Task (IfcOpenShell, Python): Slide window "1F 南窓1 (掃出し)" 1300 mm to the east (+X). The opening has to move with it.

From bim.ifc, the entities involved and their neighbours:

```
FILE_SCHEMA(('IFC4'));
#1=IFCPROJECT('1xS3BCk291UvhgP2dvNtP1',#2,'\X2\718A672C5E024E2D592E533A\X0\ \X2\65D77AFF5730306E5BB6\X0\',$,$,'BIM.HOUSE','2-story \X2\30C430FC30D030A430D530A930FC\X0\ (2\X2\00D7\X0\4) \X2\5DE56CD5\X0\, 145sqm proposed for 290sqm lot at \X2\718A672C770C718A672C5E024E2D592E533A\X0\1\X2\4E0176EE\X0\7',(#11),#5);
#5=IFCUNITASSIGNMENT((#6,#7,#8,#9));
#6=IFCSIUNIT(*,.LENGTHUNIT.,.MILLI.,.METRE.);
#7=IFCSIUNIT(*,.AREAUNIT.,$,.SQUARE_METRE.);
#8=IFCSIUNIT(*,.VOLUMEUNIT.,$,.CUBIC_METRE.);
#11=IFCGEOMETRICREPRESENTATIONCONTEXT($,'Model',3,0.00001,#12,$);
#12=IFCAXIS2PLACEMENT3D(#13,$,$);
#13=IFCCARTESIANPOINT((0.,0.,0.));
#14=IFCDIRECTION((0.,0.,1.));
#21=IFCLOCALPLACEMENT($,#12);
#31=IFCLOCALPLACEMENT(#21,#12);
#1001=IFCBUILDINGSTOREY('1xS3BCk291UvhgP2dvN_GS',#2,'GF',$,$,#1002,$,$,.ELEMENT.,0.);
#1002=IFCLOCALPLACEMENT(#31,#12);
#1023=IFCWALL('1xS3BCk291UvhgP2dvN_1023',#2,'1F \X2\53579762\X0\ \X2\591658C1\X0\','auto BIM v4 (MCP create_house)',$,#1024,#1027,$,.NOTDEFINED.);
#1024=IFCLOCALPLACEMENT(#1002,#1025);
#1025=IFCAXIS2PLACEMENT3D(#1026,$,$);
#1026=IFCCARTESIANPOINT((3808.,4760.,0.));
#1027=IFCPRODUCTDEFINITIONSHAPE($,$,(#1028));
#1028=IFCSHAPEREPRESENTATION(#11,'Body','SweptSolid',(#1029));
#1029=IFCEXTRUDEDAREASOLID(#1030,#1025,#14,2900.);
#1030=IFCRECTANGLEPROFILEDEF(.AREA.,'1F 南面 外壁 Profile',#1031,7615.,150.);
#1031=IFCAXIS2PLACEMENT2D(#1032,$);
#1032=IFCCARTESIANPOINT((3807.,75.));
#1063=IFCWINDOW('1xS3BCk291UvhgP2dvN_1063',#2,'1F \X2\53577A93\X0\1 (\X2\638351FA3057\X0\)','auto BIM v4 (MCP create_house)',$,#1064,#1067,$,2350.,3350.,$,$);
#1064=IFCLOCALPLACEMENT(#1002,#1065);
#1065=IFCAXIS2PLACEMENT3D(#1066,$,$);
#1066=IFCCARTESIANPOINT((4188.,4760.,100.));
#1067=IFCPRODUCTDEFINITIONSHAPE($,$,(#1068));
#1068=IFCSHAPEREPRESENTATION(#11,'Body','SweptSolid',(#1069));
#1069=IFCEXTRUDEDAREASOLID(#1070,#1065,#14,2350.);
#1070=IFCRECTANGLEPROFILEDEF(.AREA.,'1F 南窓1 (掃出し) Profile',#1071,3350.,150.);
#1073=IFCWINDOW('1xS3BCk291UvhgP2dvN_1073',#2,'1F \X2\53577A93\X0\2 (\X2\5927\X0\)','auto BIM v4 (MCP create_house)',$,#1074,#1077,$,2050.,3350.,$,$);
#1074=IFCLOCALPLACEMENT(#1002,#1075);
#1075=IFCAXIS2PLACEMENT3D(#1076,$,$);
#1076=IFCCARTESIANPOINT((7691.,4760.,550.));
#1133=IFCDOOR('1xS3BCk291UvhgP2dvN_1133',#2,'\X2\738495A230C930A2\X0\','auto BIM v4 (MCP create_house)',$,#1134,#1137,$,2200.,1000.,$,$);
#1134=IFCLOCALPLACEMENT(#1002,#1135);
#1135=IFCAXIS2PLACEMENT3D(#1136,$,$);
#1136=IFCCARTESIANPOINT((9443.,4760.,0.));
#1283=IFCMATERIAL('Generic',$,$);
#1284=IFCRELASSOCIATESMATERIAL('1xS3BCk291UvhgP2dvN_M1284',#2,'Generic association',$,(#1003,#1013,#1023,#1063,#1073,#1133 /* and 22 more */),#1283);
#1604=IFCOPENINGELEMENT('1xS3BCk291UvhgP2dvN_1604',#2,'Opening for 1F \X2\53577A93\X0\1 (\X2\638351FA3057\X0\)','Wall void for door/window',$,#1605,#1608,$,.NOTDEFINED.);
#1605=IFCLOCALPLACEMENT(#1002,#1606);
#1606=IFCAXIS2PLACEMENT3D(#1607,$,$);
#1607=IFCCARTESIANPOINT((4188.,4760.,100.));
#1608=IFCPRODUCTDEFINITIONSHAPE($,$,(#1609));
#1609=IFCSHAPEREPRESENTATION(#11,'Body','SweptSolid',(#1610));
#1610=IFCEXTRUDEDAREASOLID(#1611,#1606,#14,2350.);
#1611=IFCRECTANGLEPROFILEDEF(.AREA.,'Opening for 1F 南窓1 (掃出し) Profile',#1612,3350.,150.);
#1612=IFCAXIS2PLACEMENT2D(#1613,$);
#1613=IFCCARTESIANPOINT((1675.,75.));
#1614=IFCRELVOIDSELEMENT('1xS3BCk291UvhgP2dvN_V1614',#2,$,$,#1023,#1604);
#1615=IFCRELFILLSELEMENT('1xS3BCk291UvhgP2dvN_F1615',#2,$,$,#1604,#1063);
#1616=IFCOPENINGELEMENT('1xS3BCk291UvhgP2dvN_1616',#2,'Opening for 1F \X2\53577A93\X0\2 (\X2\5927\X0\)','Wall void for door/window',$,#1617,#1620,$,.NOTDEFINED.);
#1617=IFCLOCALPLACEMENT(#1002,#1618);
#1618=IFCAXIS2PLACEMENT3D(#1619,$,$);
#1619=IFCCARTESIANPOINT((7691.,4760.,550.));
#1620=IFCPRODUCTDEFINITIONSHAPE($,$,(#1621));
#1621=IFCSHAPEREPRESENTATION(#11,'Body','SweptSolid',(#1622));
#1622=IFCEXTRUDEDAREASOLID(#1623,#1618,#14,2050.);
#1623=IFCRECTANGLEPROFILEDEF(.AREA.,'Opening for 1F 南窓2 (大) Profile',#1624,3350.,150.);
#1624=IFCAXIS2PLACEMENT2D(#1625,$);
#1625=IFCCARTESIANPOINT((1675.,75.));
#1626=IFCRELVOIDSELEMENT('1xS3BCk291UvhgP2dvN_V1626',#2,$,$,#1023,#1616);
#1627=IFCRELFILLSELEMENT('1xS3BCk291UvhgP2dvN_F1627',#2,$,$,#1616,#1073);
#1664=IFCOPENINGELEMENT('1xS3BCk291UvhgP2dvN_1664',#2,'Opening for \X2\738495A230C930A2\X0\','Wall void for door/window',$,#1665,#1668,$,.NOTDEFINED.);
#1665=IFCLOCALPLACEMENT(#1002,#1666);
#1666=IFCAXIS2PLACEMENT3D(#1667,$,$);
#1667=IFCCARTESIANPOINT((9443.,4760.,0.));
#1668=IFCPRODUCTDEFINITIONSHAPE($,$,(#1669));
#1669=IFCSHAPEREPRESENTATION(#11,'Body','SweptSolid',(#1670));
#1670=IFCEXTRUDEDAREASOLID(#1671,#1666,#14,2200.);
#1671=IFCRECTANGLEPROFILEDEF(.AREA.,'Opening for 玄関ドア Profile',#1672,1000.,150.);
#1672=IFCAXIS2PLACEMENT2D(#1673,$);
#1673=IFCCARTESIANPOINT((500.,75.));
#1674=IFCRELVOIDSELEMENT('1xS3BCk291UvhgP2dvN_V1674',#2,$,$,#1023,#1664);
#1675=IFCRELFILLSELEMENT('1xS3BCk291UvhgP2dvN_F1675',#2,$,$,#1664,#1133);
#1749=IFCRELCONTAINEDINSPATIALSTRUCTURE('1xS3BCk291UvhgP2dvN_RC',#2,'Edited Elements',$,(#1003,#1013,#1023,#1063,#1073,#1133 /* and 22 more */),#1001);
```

```python
import ifcopenshell
import ifcopenshell.api.geometry
import ifcopenshell.util.placement

model = ifcopenshell.open("bim.ifc")

window = model.by_id(1063)
opening = window.FillsVoids[0].RelatingOpeningElement
wall = opening.VoidsElements[0].RelatingBuildingElement

wall_matrix = ifcopenshell.util.placement.get_local_placement(wall.ObjectPlacement)
shift = wall_matrix[:3, 0] * 1300.0
before = ifcopenshell.util.placement.get_local_placement(window.ObjectPlacement)[:3, 3].copy()

# The window is not placed relative to its opening, so move both.
for product in (opening, window):
    matrix = ifcopenshell.util.placement.get_local_placement(product.ObjectPlacement)
    matrix[:3, 3] += shift
    ifcopenshell.api.geometry.edit_object_placement(model, product=product, matrix=matrix, is_si=False)

after = ifcopenshell.util.placement.get_local_placement(window.ObjectPlacement)[:3, 3]
print("window moved by", (after - before).round(3) + 0.0)

model.write("bim_rev.ifc")
```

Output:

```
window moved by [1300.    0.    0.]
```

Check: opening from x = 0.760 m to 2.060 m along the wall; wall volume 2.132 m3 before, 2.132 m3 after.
